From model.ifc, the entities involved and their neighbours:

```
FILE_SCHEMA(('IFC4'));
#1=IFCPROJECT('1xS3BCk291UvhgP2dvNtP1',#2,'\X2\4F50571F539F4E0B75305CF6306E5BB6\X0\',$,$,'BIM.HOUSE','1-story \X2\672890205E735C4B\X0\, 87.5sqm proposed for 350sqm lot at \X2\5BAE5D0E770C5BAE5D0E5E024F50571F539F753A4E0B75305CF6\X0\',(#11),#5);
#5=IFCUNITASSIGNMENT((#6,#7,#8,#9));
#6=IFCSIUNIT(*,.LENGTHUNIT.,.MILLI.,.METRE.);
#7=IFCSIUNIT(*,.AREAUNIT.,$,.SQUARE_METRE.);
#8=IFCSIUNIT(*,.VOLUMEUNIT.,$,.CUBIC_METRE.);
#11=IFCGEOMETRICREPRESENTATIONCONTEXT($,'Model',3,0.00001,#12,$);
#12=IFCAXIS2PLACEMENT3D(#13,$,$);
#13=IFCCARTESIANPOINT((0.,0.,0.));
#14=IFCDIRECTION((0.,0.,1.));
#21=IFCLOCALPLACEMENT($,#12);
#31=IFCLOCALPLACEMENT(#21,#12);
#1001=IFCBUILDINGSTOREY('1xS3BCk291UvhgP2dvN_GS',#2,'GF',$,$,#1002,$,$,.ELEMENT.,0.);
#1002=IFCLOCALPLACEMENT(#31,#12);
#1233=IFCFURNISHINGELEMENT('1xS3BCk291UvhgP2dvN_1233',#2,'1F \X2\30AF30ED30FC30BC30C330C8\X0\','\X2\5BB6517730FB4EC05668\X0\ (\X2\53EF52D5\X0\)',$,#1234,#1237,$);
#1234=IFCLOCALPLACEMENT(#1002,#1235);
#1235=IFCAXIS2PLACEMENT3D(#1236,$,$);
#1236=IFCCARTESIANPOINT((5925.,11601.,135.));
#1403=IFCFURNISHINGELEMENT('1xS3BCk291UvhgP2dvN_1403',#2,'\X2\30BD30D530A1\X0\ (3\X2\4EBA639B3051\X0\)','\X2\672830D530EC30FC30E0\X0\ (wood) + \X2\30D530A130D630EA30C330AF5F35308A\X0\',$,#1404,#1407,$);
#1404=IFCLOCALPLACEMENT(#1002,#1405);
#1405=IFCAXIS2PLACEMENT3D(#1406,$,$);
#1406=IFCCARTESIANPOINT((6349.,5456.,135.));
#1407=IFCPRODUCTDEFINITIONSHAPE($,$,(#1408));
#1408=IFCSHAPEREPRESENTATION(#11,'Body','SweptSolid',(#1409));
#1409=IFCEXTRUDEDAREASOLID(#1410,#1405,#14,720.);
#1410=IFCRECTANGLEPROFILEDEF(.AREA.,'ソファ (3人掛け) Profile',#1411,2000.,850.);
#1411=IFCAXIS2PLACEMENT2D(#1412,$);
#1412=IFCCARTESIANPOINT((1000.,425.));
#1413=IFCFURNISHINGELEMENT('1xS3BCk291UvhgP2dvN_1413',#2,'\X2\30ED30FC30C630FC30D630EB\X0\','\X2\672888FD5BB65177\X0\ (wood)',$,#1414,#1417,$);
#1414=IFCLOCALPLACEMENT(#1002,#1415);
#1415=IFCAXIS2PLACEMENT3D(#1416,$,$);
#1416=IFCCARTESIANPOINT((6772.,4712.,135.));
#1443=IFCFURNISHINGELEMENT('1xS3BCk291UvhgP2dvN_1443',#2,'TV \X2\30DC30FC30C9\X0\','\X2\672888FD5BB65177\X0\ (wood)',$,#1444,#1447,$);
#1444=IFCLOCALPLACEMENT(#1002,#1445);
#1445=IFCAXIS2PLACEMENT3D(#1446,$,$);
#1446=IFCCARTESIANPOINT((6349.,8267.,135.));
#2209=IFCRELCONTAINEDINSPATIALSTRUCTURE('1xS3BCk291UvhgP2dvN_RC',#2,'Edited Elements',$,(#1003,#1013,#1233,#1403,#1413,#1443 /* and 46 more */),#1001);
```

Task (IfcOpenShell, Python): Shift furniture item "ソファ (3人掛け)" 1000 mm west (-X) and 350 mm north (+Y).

```python
import ifcopenshell
import ifcopenshell.api.geometry
import ifcopenshell.util.placement
import ifcopenshell.util.unit

model = ifcopenshell.open("model.ifc")
unit_scale = ifcopenshell.util.unit.calculate_unit_scale(model)

item = model.by_id(1403)
matrix = ifcopenshell.util.placement.get_local_placement(item.ObjectPlacement)
matrix[0, 3] -= 1 / unit_scale
matrix[1, 3] += 0.35 / unit_scale
ifcopenshell.api.geometry.edit_object_placement(model, product=item, matrix=matrix, is_si=False)

print(ifcopenshell.util.placement.get_local_placement(item.ObjectPlacement).round(3) + 0.0)

model.write("model_rev.ifc")
```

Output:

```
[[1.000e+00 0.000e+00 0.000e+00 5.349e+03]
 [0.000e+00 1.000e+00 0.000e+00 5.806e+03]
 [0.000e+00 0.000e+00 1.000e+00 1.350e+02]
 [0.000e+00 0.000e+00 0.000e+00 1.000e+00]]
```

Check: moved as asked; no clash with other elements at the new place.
